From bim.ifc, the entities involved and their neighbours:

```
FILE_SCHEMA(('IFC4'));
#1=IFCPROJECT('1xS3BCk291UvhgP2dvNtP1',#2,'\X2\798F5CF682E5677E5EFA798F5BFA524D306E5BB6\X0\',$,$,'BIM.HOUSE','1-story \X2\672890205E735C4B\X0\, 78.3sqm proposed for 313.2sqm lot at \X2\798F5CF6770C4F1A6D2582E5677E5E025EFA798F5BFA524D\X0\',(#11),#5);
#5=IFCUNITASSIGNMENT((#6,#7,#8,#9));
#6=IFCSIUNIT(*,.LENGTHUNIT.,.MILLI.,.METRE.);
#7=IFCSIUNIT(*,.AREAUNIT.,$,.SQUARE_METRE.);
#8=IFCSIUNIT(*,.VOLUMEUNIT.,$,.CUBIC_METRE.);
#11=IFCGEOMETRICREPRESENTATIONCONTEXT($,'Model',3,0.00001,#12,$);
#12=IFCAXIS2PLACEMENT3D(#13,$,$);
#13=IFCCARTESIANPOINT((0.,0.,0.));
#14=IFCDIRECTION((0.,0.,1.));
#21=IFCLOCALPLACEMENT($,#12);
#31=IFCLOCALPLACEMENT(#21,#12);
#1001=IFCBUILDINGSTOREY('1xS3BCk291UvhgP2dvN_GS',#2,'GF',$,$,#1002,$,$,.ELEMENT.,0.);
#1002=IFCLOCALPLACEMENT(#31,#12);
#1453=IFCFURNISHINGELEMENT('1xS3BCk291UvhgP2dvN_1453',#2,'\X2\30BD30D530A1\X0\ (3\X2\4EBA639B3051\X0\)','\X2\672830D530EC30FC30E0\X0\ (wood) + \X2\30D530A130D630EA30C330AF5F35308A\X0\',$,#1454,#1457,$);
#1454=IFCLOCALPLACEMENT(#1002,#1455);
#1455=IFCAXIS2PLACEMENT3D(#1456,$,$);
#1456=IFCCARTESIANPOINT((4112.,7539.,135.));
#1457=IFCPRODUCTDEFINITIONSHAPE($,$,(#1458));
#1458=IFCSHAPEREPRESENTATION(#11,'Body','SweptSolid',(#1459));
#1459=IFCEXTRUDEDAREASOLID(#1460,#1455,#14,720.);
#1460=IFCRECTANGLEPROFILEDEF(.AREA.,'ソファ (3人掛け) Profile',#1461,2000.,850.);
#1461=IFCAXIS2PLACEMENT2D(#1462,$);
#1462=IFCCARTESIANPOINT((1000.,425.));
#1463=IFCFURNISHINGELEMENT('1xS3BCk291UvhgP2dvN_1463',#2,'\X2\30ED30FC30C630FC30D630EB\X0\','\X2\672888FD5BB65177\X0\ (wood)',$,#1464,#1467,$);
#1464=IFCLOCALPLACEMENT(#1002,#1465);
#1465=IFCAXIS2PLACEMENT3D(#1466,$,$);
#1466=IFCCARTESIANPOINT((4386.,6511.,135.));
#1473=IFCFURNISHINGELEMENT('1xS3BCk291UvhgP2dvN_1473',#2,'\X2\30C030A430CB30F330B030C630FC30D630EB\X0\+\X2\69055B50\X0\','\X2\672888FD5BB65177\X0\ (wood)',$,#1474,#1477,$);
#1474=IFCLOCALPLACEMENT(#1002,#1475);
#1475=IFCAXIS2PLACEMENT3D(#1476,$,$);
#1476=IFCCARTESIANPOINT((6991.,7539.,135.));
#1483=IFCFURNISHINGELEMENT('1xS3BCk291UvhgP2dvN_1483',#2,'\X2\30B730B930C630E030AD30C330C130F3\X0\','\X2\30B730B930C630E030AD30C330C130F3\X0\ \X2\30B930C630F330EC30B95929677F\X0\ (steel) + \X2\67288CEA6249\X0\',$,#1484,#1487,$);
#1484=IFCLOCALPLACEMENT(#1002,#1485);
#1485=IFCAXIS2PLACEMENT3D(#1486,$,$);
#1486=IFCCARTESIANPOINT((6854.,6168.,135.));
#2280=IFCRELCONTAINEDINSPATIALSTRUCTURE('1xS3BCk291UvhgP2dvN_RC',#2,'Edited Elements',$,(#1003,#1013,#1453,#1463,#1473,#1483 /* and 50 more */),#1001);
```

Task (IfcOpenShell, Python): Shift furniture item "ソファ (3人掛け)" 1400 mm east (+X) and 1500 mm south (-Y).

```python
import ifcopenshell
import ifcopenshell.api.geometry
import ifcopenshell.util.placement

model = ifcopenshell.open("bim.ifc")

item = model.by_id(1453)
matrix = ifcopenshell.util.placement.get_local_placement(item.ObjectPlacement)
matrix[0, 3] += 1400.0
matrix[1, 3] -= 1500.0
ifcopenshell.api.geometry.edit_object_placement(model, product=item, matrix=matrix, is_si=False)

print(ifcopenshell.util.placement.get_local_placement(item.ObjectPlacement).round(3) + 0.0)

model.write("bim_edited.ifc")
```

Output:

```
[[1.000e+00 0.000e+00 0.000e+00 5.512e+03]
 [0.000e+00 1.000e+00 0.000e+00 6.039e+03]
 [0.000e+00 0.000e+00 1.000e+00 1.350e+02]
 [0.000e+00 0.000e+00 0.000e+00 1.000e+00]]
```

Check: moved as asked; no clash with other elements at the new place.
